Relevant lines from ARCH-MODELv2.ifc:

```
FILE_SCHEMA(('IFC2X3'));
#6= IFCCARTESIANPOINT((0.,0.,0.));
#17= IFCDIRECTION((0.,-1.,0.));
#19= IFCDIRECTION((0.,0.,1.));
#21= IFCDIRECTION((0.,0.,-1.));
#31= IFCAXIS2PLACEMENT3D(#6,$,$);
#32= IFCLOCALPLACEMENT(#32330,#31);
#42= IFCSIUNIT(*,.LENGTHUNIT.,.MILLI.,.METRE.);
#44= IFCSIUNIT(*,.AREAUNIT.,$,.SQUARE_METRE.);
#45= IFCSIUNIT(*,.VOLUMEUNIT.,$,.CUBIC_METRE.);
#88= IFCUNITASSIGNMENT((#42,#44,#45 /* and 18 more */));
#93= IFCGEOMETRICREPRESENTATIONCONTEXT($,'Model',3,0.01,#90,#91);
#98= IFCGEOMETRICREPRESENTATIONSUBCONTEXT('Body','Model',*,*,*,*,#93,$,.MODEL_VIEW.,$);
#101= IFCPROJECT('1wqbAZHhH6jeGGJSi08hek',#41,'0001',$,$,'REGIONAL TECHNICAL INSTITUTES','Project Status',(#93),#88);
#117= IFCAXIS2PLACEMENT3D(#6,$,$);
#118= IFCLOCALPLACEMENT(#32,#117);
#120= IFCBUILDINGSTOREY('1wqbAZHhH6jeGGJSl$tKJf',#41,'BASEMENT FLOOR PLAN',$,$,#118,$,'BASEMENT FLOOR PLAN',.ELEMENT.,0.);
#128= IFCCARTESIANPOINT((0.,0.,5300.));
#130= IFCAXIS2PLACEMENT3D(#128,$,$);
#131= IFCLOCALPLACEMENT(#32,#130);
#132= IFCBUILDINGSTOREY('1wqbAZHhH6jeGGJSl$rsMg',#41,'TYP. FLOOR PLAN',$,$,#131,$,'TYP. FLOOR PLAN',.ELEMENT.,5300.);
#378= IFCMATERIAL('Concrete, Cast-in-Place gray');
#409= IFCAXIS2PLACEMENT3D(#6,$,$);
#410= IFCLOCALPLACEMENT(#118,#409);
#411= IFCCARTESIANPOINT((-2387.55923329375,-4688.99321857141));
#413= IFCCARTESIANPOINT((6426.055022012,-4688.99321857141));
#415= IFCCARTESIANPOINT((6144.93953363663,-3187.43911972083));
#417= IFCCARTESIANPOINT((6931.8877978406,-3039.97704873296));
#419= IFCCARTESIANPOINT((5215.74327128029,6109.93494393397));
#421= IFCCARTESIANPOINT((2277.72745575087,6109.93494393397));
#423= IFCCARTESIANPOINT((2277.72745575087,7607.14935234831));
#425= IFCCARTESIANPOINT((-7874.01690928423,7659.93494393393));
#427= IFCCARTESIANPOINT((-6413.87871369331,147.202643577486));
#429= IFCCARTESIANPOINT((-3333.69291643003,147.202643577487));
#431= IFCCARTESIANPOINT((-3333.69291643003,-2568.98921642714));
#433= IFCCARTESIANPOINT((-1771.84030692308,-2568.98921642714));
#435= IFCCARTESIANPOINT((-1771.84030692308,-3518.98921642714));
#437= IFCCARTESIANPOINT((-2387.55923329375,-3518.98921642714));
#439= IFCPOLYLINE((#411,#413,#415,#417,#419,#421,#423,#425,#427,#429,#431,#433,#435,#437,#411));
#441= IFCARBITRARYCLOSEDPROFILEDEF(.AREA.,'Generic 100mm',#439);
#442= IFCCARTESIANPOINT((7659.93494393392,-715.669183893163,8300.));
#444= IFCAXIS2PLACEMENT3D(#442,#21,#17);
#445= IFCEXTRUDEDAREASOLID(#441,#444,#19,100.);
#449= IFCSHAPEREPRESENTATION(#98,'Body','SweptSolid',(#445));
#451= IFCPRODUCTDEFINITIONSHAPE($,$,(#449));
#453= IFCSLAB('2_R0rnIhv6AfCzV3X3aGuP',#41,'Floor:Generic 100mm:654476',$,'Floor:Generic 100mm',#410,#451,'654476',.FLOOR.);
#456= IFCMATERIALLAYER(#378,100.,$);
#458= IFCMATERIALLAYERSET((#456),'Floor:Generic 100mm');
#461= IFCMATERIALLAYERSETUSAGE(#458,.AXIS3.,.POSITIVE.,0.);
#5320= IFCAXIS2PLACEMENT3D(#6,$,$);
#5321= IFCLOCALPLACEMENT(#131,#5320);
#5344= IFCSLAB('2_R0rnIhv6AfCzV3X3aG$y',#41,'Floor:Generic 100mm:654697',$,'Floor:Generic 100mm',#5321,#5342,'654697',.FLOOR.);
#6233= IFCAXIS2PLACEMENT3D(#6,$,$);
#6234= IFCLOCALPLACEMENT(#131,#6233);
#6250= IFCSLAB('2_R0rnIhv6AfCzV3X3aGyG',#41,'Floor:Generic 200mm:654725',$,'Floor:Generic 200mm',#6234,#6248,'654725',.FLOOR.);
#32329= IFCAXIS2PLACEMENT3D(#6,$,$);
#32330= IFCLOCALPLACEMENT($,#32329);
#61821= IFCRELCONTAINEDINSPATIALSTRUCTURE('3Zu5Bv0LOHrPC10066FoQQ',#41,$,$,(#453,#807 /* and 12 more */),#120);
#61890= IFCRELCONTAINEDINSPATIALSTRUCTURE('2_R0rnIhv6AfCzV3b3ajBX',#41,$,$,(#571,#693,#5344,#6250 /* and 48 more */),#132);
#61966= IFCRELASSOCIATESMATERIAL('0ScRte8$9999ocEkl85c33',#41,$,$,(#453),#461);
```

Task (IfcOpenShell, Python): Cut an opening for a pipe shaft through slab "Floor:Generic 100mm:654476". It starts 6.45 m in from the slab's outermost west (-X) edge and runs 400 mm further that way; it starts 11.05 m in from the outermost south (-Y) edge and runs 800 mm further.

```python
import numpy as np
import ifcopenshell
import ifcopenshell.api.feature
import ifcopenshell.api.geometry
import ifcopenshell.api.root
import ifcopenshell.geom
import ifcopenshell.util.placement
import ifcopenshell.util.representation
import ifcopenshell.util.shape
import ifcopenshell.util.unit

model = ifcopenshell.open("ARCH-MODELv2.ifc")
unit_scale = ifcopenshell.util.unit.calculate_unit_scale(model)
settings = ifcopenshell.geom.settings()


def volume(element):
    """Net volume in cubic metres, openings subtracted."""
    shape = ifcopenshell.geom.create_shape(settings, element)
    return ifcopenshell.util.shape.get_volume(shape.geometry)


slab = model.by_id(453)
before = volume(slab)

# Extent in the slab's own axes, in metres. The edges named are its -X and -Y sides.
slab_shape = ifcopenshell.geom.create_shape(settings, slab)
vertices = ifcopenshell.util.shape.get_vertices(slab_shape.geometry)
x_min, y_min, bottom = vertices.min(axis=0)
top = vertices[:, 2].max()

opening = ifcopenshell.api.root.create_entity(model, ifc_class="IfcOpeningElement", name="Pipe shaft opening")
context = ifcopenshell.util.representation.get_context(model, "Model", "Body", "MODEL_VIEW")
width, depth = 0.4, 0.8
outline = [(0.0, 0.0), (width, 0.0), (width, depth), (0.0, depth), (0.0, 0.0)]
# Overshoot both faces by 50 mm so the cut is clean.
shape = ifcopenshell.api.geometry.add_slab_representation(
    model, context=context, depth=top - bottom + 0.1, polyline=outline
)
ifcopenshell.api.geometry.assign_representation(model, product=opening, representation=shape)

matrix = ifcopenshell.util.placement.get_local_placement(slab.ObjectPlacement)
matrix[:, 3] = matrix @ np.append(np.array([x_min + 6.45, y_min + 11.05, bottom - 0.05]) / unit_scale, 1.0)
ifcopenshell.api.geometry.edit_object_placement(model, product=opening, matrix=matrix, is_si=False)
ifcopenshell.api.feature.add_feature(model, feature=opening, element=slab)

after = volume(slab)

print(f"slab volume {before:.3f} -> {after:.3f} m3")

model.write("ARCH-MODELv2_rev.ifc")
```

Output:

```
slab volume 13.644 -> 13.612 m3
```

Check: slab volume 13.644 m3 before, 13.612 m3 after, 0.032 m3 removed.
